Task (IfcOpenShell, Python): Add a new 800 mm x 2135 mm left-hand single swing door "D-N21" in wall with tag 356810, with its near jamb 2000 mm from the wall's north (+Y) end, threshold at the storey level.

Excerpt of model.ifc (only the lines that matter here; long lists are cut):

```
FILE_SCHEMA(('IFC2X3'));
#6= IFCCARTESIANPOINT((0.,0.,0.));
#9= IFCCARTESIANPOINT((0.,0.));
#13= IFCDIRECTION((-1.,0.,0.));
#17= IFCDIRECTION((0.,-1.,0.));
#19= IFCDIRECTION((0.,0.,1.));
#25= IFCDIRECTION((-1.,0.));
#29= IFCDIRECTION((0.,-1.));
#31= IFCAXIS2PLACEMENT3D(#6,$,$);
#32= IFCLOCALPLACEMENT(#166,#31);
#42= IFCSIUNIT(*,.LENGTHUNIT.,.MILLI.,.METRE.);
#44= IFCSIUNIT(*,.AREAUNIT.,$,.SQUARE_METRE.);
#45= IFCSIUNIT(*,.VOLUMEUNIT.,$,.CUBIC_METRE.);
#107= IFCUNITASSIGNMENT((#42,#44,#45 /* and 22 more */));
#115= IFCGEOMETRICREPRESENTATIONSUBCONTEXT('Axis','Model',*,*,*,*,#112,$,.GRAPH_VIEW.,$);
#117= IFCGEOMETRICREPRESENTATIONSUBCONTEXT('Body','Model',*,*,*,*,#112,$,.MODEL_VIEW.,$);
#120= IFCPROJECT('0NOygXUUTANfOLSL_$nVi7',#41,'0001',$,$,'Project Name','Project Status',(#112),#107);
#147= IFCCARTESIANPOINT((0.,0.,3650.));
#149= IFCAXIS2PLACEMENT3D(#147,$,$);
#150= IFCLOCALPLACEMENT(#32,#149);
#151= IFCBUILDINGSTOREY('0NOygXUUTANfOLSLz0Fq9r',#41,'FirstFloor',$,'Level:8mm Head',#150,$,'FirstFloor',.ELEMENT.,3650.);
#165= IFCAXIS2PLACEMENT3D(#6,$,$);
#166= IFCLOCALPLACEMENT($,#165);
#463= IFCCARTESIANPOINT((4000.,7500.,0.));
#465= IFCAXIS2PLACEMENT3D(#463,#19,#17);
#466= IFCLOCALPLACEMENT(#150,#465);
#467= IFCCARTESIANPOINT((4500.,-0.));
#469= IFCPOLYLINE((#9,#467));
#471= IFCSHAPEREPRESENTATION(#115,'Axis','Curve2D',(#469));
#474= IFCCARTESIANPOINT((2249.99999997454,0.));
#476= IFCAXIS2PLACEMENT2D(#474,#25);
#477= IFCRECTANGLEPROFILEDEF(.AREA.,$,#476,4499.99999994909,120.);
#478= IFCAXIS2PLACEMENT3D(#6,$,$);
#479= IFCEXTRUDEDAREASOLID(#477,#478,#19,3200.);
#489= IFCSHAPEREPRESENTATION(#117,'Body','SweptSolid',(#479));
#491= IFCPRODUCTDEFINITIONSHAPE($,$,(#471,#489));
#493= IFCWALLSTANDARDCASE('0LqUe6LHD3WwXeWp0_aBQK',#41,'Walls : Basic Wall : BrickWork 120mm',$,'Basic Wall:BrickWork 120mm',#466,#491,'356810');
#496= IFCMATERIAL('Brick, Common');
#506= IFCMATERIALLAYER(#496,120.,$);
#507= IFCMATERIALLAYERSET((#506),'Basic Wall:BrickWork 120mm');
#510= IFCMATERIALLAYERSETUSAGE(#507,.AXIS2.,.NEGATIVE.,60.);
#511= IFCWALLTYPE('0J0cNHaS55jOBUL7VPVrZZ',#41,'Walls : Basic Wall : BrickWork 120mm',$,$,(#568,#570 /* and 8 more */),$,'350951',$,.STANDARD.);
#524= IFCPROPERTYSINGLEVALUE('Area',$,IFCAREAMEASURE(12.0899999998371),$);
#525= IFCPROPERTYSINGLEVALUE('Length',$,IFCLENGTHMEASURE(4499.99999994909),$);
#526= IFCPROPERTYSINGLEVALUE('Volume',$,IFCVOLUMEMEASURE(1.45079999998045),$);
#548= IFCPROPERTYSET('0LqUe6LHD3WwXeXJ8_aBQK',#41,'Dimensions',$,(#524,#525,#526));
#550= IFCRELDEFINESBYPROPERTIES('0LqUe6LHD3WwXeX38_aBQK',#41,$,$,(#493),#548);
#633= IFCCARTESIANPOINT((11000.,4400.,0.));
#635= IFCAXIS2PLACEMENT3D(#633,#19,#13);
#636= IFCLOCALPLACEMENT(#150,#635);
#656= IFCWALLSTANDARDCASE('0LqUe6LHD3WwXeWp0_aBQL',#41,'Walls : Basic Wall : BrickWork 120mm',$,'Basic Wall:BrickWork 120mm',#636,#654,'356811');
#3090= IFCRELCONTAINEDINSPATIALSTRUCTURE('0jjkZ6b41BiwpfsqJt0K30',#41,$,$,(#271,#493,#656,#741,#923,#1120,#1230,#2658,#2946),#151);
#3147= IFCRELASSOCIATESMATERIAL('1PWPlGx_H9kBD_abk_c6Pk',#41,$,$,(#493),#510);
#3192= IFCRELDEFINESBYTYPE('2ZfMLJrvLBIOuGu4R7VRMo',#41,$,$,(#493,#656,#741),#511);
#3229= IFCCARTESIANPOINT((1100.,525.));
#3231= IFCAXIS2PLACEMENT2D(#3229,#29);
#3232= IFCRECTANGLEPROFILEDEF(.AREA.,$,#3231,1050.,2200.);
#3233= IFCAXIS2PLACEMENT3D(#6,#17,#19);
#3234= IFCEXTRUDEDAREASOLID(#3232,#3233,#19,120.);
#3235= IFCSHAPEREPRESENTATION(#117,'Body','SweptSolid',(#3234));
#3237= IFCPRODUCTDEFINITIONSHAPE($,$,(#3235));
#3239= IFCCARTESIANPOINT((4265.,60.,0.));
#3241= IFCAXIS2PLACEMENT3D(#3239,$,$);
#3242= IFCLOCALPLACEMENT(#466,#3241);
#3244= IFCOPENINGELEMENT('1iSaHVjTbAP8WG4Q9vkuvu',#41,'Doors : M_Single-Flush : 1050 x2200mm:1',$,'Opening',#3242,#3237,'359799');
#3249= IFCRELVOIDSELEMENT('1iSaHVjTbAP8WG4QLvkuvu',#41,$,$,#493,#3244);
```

```python
import numpy as np
import ifcopenshell
import ifcopenshell.api.feature
import ifcopenshell.api.geometry
import ifcopenshell.api.pset
import ifcopenshell.api.root
import ifcopenshell.api.spatial
import ifcopenshell.api.type
import ifcopenshell.geom
import ifcopenshell.util.element
import ifcopenshell.util.placement
import ifcopenshell.util.representation
import ifcopenshell.util.shape
import ifcopenshell.util.unit

model = ifcopenshell.open("model.ifc")
unit_scale = ifcopenshell.util.unit.calculate_unit_scale(model)
area_scale = ifcopenshell.util.unit.calculate_unit_scale(model, "AREAUNIT")
volume_scale = ifcopenshell.util.unit.calculate_unit_scale(model, "VOLUMEUNIT")
settings = ifcopenshell.geom.settings()


def volume(element):
    """Net volume in cubic metres, openings subtracted."""
    shape = ifcopenshell.geom.create_shape(settings, element)
    return ifcopenshell.util.shape.get_volume(shape.geometry)


wall = model.by_guid("0LqUe6LHD3WwXeWp0_aBQK")
storey = ifcopenshell.util.element.get_container(wall, ifc_class="IfcBuildingStorey")
context = ifcopenshell.util.representation.get_context(model, "Model", "Body", "MODEL_VIEW")
before = volume(wall)

width, height, from_end, sill = 0.8, 2.135, 2, 0.0  # metres

# The wall runs along its own X axis, and the end named is its -X end.
wall_shape = ifcopenshell.geom.create_shape(settings, wall)
x, y, z = ifcopenshell.util.shape.get_vertices(wall_shape.geometry).T
start = x.min() + from_end
face, thickness = float(y.min()), float(y.max() - y.min())
wall_matrix = ifcopenshell.util.placement.get_local_placement(wall.ObjectPlacement)
level = ifcopenshell.util.placement.get_local_placement(storey.ObjectPlacement)[2, 3]


def in_wall(x, y):
    """Placement at x, y metres in the wall's axes, at sill height."""
    matrix = wall_matrix.copy()
    matrix[:, 3] = wall_matrix @ np.array([x / unit_scale, y / unit_scale, 0.0, 1.0])
    matrix[2, 3] = level + sill / unit_scale
    return matrix


# Opening: a box that overshoots both wall faces by 50 mm.
opening = ifcopenshell.api.root.create_entity(model, ifc_class="IfcOpeningElement")
box = ifcopenshell.api.geometry.add_wall_representation(
    model, context=context, length=width, height=height, thickness=thickness + 0.1
)
ifcopenshell.api.geometry.assign_representation(model, product=opening, representation=box)
ifcopenshell.api.geometry.edit_object_placement(model, product=opening, matrix=in_wall(start, face - 0.05), is_si=False)
ifcopenshell.api.feature.add_feature(model, feature=opening, element=wall)

door = ifcopenshell.api.root.create_entity(model, ifc_class="IfcDoor", name="D-N21")
door.OverallWidth, door.OverallHeight = width / unit_scale, height / unit_scale
body = ifcopenshell.api.geometry.add_door_representation(
    model,
    context=context,
    overall_width=door.OverallWidth,
    overall_height=door.OverallHeight,
    operation_type="SINGLE_SWING_LEFT",
    lining_properties={"LiningDepth": thickness / unit_scale, "ThresholdDepth": thickness / unit_scale},
)
ifcopenshell.api.geometry.assign_representation(model, product=door, representation=body)
ifcopenshell.api.spatial.assign_container(model, products=[door], relating_structure=storey)
fills = ifcopenshell.api.feature.add_filling(model, opening=opening, element=door)
fills.OwnerHistory = door.OwnerHistory  # required in IFC2X3

# IFC2X3 keeps the operation on the door style.
style = ifcopenshell.api.root.create_entity(model, ifc_class="IfcDoorStyle", name="D-N21")
style.OperationType, style.ConstructionType = "SINGLE_SWING_LEFT", "NOTDEFINED"
style.ParameterTakesPrecedence = style.Sizeable = False
ifcopenshell.api.type.assign_type(model, related_objects=[door], relating_type=style)

# The lining spans the wall, so the door starts at the wall face.
ifcopenshell.api.geometry.edit_object_placement(model, product=door, matrix=in_wall(start, face), is_si=False)

after = volume(wall)

# Update the wall's stored quantities.
pset = model.by_id(ifcopenshell.util.element.get_pset(wall, "Dimensions", should_inherit=False)["id"])
ifcopenshell.api.pset.edit_pset(model, pset=pset, properties={
    "Area": model.create_entity("IfcAreaMeasure", after / thickness / area_scale),
    "Volume": model.create_entity("IfcVolumeMeasure", after / volume_scale),
})

print(f"wall volume {before:.3f} -> {after:.3f} m3")

model.write("model_updated.ifc")
```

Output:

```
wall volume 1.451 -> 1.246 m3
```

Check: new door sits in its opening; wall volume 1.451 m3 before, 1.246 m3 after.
